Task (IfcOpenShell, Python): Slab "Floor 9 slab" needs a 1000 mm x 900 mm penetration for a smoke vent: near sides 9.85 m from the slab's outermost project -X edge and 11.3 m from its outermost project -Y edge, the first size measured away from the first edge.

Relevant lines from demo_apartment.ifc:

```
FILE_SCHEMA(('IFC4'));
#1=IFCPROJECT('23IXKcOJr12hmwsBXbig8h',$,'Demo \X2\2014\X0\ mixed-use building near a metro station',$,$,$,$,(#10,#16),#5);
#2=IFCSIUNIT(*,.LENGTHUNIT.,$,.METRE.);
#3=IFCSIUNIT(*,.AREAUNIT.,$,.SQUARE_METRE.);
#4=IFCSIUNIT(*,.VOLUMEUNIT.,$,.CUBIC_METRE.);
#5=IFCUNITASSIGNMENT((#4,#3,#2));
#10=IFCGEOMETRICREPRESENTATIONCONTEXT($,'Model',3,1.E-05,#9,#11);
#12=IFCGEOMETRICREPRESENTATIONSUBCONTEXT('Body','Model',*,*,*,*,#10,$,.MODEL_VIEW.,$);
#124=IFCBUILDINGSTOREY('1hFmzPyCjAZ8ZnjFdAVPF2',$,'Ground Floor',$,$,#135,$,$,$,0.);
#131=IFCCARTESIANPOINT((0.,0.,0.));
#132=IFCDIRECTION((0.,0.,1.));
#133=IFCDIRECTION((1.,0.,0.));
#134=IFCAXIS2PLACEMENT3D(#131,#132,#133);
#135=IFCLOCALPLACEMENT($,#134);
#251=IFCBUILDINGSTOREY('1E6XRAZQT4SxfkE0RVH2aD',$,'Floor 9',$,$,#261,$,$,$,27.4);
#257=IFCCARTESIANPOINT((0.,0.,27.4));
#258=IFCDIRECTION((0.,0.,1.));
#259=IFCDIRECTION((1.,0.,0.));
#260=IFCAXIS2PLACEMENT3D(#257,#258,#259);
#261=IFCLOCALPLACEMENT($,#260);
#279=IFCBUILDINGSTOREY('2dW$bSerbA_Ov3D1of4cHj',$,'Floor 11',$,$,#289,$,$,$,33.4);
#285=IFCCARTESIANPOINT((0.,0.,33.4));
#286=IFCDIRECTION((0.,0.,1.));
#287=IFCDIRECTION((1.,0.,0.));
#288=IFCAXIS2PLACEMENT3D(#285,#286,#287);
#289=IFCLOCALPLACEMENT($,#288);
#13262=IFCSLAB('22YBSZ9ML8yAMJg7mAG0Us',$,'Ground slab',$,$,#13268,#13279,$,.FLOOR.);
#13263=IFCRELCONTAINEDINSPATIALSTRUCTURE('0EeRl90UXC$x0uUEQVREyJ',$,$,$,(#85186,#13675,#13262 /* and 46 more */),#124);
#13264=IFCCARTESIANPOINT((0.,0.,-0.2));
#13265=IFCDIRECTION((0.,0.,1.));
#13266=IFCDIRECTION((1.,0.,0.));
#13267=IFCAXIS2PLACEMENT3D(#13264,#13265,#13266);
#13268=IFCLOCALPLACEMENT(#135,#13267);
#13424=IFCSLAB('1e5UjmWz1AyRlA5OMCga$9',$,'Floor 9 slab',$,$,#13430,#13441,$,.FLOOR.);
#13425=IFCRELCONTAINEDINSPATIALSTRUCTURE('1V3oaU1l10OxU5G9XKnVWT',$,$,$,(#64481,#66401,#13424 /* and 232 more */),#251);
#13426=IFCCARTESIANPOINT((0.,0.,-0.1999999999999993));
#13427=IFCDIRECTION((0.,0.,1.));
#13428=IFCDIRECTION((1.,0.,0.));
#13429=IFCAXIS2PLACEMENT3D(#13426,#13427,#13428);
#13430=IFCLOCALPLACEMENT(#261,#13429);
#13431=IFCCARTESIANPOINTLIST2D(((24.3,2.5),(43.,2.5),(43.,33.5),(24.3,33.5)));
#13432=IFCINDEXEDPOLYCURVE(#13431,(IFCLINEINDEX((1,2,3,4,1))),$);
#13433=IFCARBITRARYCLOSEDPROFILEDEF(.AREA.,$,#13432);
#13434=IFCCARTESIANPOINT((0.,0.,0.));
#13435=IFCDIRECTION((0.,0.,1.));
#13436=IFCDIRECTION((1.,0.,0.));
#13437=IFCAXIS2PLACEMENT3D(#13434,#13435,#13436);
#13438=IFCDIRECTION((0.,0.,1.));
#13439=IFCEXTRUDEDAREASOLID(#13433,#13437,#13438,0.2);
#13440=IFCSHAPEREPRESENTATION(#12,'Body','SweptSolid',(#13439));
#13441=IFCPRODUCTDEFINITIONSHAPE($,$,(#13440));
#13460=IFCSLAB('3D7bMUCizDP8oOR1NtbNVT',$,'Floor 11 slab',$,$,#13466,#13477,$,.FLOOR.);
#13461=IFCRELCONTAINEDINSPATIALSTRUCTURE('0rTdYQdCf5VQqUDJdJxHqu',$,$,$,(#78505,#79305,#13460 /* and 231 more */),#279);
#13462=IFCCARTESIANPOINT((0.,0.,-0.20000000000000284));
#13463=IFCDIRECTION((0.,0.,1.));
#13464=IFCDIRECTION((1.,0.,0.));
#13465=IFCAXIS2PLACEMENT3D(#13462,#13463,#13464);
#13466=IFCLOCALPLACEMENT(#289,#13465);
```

```python
import numpy as np
import ifcopenshell
import ifcopenshell.api.feature
import ifcopenshell.api.geometry
import ifcopenshell.api.root
import ifcopenshell.geom
import ifcopenshell.util.placement
import ifcopenshell.util.representation
import ifcopenshell.util.shape
import ifcopenshell.util.unit

model = ifcopenshell.open("demo_apartment.ifc")
unit_scale = ifcopenshell.util.unit.calculate_unit_scale(model)
settings = ifcopenshell.geom.settings()


def volume(element):
    """Net volume in cubic metres, openings subtracted."""
    shape = ifcopenshell.geom.create_shape(settings, element)
    return ifcopenshell.util.shape.get_volume(shape.geometry)


slab = model.by_guid("1e5UjmWz1AyRlA5OMCga$9")
before = volume(slab)

# Extent in the slab's own axes, in metres. The edges named are its -X and -Y sides.
slab_shape = ifcopenshell.geom.create_shape(settings, slab)
vertices = ifcopenshell.util.shape.get_vertices(slab_shape.geometry)
x_min, y_min, bottom = vertices.min(axis=0)
top = vertices[:, 2].max()

opening = ifcopenshell.api.root.create_entity(model, ifc_class="IfcOpeningElement", name="Smoke vent opening", predefined_type="OPENING")
context = ifcopenshell.util.representation.get_context(model, "Model", "Body", "MODEL_VIEW")
width, depth = 1, 0.9
outline = [(0.0, 0.0), (width, 0.0), (width, depth), (0.0, depth), (0.0, 0.0)]
# Overshoot both faces by 50 mm so the cut is clean.
shape = ifcopenshell.api.geometry.add_slab_representation(
    model, context=context, depth=top - bottom + 0.1, polyline=outline
)
ifcopenshell.api.geometry.assign_representation(model, product=opening, representation=shape)

matrix = ifcopenshell.util.placement.get_local_placement(slab.ObjectPlacement)
matrix[:, 3] = matrix @ np.append(np.array([x_min + 9.85, y_min + 11.3, bottom - 0.05]) / unit_scale, 1.0)
ifcopenshell.api.geometry.edit_object_placement(model, product=opening, matrix=matrix, is_si=False)
ifcopenshell.api.feature.add_feature(model, feature=opening, element=slab)

after = volume(slab)

print(f"slab volume {before:.3f} -> {after:.3f} m3")

model.write("demo_apartment_v2.ifc")
```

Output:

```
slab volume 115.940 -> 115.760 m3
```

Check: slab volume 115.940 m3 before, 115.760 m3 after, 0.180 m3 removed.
